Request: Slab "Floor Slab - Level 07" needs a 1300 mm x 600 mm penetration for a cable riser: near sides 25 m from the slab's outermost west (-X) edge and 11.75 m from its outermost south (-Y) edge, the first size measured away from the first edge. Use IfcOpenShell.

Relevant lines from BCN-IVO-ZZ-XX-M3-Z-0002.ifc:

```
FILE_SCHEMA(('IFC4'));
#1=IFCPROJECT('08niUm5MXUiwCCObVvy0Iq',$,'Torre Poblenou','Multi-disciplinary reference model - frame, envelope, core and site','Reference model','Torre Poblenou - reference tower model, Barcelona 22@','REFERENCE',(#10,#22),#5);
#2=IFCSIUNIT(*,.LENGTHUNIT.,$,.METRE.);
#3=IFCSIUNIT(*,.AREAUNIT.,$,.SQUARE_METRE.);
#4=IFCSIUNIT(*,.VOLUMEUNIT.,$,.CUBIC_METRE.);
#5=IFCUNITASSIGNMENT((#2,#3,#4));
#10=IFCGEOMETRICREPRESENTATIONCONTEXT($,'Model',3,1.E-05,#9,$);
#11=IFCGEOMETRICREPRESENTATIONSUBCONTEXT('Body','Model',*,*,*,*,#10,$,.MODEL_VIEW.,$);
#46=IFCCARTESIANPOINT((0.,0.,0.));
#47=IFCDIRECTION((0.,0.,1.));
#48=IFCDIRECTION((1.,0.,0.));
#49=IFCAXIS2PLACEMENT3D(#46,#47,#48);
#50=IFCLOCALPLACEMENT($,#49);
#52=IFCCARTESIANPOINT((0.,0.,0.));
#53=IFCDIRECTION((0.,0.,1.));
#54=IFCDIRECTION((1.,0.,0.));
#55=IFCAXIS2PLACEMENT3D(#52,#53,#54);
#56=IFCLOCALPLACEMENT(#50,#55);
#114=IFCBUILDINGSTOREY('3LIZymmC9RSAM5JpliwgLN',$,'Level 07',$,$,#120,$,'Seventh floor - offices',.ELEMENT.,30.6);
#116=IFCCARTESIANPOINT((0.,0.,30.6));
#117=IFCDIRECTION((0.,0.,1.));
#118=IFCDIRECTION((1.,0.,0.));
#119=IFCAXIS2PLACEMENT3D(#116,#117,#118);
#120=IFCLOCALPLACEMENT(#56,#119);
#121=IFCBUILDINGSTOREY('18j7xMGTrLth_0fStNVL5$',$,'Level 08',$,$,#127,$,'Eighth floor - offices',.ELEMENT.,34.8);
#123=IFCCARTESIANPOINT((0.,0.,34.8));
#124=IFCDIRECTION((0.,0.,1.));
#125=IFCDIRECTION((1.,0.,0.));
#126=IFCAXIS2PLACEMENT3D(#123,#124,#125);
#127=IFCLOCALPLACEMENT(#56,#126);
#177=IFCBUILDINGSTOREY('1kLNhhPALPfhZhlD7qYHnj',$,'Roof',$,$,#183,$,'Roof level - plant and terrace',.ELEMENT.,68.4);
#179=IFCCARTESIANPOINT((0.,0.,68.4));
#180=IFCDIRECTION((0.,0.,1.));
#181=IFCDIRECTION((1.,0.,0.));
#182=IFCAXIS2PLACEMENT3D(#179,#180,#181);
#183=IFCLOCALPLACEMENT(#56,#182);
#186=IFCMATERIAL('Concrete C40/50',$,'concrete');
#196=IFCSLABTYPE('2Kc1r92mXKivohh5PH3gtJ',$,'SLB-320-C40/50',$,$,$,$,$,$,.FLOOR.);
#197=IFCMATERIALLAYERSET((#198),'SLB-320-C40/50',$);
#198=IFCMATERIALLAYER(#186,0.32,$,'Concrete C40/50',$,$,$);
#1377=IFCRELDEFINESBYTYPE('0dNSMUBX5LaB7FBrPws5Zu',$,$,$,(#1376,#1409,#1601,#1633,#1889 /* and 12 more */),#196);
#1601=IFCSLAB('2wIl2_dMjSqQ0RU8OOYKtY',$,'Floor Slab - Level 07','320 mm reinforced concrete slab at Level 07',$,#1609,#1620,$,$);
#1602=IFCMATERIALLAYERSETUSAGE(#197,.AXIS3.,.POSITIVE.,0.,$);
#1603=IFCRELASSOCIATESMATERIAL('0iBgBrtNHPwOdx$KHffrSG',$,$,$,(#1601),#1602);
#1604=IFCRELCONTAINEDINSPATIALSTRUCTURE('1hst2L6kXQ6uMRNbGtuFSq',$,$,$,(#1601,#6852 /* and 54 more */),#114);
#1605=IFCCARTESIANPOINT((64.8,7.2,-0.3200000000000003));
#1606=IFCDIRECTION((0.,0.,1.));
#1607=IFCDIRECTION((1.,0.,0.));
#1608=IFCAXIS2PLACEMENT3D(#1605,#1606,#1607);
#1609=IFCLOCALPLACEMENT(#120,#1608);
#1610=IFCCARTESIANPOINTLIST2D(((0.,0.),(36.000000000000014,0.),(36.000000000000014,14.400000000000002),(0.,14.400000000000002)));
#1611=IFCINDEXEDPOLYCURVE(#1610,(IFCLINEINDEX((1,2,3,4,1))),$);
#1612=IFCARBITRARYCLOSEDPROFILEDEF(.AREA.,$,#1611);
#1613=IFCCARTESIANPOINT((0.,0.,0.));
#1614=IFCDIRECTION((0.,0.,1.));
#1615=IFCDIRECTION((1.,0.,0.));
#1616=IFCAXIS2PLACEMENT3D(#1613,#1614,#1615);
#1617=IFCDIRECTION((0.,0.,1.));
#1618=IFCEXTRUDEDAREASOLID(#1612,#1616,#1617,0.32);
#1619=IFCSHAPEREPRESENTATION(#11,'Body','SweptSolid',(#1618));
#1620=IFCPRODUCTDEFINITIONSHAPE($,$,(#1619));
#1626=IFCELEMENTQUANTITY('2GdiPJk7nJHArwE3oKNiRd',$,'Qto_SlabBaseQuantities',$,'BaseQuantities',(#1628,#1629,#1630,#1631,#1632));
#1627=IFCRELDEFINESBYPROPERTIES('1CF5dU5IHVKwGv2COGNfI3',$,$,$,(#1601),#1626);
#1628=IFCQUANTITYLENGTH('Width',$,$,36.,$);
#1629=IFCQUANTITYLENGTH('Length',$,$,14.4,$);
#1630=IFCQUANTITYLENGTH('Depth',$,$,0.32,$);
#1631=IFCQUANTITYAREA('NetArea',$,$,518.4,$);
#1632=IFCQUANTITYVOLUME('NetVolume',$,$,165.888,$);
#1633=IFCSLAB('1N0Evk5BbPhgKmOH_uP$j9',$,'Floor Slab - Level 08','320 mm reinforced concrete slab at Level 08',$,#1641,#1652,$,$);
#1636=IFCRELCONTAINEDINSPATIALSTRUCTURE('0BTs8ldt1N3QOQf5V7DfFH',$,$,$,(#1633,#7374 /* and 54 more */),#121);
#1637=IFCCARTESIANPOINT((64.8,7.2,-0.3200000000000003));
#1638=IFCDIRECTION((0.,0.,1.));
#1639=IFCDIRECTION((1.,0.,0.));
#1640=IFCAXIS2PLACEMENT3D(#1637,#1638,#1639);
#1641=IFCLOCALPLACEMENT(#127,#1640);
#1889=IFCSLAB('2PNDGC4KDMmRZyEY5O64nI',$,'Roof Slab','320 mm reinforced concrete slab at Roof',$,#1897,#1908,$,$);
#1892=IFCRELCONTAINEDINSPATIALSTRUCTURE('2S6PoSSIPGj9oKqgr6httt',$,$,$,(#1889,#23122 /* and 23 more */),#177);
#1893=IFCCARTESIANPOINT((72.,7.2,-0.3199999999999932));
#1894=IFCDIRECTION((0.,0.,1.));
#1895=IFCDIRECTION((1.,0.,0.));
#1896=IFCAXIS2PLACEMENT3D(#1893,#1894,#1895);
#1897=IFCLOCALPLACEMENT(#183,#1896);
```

```python
import numpy as np
import ifcopenshell
import ifcopenshell.api.feature
import ifcopenshell.api.geometry
import ifcopenshell.api.pset
import ifcopenshell.api.root
import ifcopenshell.geom
import ifcopenshell.util.element
import ifcopenshell.util.placement
import ifcopenshell.util.representation
import ifcopenshell.util.shape
import ifcopenshell.util.unit

model = ifcopenshell.open("BCN-IVO-ZZ-XX-M3-Z-0002.ifc")
unit_scale = ifcopenshell.util.unit.calculate_unit_scale(model)
area_scale = ifcopenshell.util.unit.calculate_unit_scale(model, "AREAUNIT")
volume_scale = ifcopenshell.util.unit.calculate_unit_scale(model, "VOLUMEUNIT")
settings = ifcopenshell.geom.settings()


def volume(element):
    """Net volume in cubic metres, openings subtracted."""
    shape = ifcopenshell.geom.create_shape(settings, element)
    return ifcopenshell.util.shape.get_volume(shape.geometry)


slab = model.by_guid("2wIl2_dMjSqQ0RU8OOYKtY")
before = volume(slab)

# Extent in the slab's own axes, in metres. The edges named are its -X and -Y sides.
slab_shape = ifcopenshell.geom.create_shape(settings, slab)
vertices = ifcopenshell.util.shape.get_vertices(slab_shape.geometry)
x_min, y_min, bottom = vertices.min(axis=0)
top = vertices[:, 2].max()

opening = ifcopenshell.api.root.create_entity(model, ifc_class="IfcOpeningElement", name="Cable riser opening", predefined_type="OPENING")
context = ifcopenshell.util.representation.get_context(model, "Model", "Body", "MODEL_VIEW")
width, depth = 1.3, 0.6
outline = [(0.0, 0.0), (width, 0.0), (width, depth), (0.0, depth), (0.0, 0.0)]
# Overshoot both faces by 50 mm so the cut is clean.
shape = ifcopenshell.api.geometry.add_slab_representation(
    model, context=context, depth=top - bottom + 0.1, polyline=outline
)
ifcopenshell.api.geometry.assign_representation(model, product=opening, representation=shape)

matrix = ifcopenshell.util.placement.get_local_placement(slab.ObjectPlacement)
matrix[:, 3] = matrix @ np.append(np.array([x_min + 25, y_min + 11.75, bottom - 0.05]) / unit_scale, 1.0)
ifcopenshell.api.geometry.edit_object_placement(model, product=opening, matrix=matrix, is_si=False)
ifcopenshell.api.feature.add_feature(model, feature=opening, element=slab)

after = volume(slab)

# Update the slab's stored quantities.
qto = model.by_id(ifcopenshell.util.element.get_pset(slab, "Qto_SlabBaseQuantities", should_inherit=False)["id"])
ifcopenshell.api.pset.edit_qto(model, qto=qto, properties={
    "NetArea": after / (top - bottom) / area_scale,
    "NetVolume": after / volume_scale,
})

print(f"slab volume {before:.3f} -> {after:.3f} m3")

model.write("BCN-IVO-ZZ-XX-M3-Z-0002-out.ifc")
```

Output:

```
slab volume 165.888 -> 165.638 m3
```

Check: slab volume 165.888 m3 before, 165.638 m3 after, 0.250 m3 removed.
